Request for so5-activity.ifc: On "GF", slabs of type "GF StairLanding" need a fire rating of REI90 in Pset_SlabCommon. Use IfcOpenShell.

First a look at what the model holds.

```python
import ifcopenshell
import ifcopenshell.util.element

model = ifcopenshell.open("so5-activity.ifc")
print(model.schema)
storey = next(s for s in model.by_type("IfcBuildingStorey") if s.Name == "GF")
slabs = [e for e in ifcopenshell.util.element.get_decomposition(storey) if e.is_a("IfcSlab")]
seen = {}
for e in slabs:
    element_type = ifcopenshell.util.element.get_type(e)
    key = (element_type.Name if element_type != e and element_type else None, ifcopenshell.util.element.get_pset(e, "Pset_SlabCommon", "FireRating"))
    seen[key] = seen.get(key, 0) + 1
for (name, value), count in sorted(seen.items(), key=str):
    print(count, "x", name, "|", value)
```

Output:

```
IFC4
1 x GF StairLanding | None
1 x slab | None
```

```python
import ifcopenshell
import ifcopenshell.api.pset
import ifcopenshell.util.element

model = ifcopenshell.open("so5-activity.ifc")

storey = next(s for s in model.by_type("IfcBuildingStorey") if s.Name == "GF")
slabs = [e for e in ifcopenshell.util.element.get_decomposition(storey) if e.is_a("IfcSlab")]

count = 0
for e in slabs:
    element_type = ifcopenshell.util.element.get_type(e)
    if element_type in (None, e) or element_type.Name != "GF StairLanding":
        continue
    # add_pset returns the element's existing set when there is one.
    pset = ifcopenshell.api.pset.add_pset(model, product=e, name="Pset_SlabCommon")
    ifcopenshell.api.pset.edit_pset(model, pset=pset, properties={"FireRating": "REI90"})
    count += 1

print(count, "slabs updated")

model.write("so5-activity-out.ifc")
```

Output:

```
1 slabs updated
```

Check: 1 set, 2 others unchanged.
